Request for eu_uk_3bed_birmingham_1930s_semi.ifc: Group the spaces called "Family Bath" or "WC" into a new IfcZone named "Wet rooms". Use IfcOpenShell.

First a look at what the model holds.

```python
import ifcopenshell

model = ifcopenshell.open("eu_uk_3bed_birmingham_1930s_semi.ifc")
print(model.schema)
seen = {}
for space in model.by_type("IfcSpace"):
    seen[space.LongName] = seen.get(space.LongName, 0) + 1
for name, count in sorted(seen.items(), key=str):
    print(count, "x", name)
print("zones:", [z.Name for z in model.by_type("IfcZone")][:20])
```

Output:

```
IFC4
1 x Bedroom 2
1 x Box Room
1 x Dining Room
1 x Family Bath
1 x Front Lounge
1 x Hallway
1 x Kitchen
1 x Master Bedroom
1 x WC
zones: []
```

```python
import ifcopenshell
import ifcopenshell.api.group
import ifcopenshell.api.root

model = ifcopenshell.open("eu_uk_3bed_birmingham_1930s_semi.ifc")

names = {"Family Bath", "WC"}
spaces = [s for s in model.by_type("IfcSpace") if s.LongName in names]

zone = ifcopenshell.api.root.create_entity(model, ifc_class="IfcZone", name="Wet rooms")
ifcopenshell.api.group.assign_group(model, products=spaces, group=zone)
print(len(spaces), "spaces in", zone.Name)

model.write("eu_uk_3bed_birmingham_1930s_semi_edited.ifc")
```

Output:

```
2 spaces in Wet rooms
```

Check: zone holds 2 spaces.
